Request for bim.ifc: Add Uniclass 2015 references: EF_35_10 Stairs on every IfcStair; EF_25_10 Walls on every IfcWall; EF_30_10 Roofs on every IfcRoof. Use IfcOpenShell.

First a look at what the model holds.

```python
import ifcopenshell

model = ifcopenshell.open("bim.ifc")
print(model.schema)
print("classifications:", [c.Name for c in model.by_type("IfcClassification")])
for ifc_class in ("IfcDoor", "IfcRoof", "IfcStair", "IfcWall", "IfcWindow"):
    print(ifc_class, len(model.by_type(ifc_class)))
```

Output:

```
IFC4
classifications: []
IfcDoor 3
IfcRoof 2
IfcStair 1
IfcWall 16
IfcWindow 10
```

```python
import ifcopenshell
import ifcopenshell.api.classification

model = ifcopenshell.open("bim.ifc")

system = ifcopenshell.api.classification.add_classification(model, classification="Uniclass 2015")

codes = {
    "IfcStair": ("EF_35_10", "Stairs"),
    "IfcWall": ("EF_25_10", "Walls"),
    "IfcRoof": ("EF_30_10", "Roofs"),
}
for ifc_class, (code, name) in codes.items():
    products = model.by_type(ifc_class)
    ifcopenshell.api.classification.add_reference(
        model, products=products, classification=system, identification=code, name=name
    )
    print(code, len(products))

model.write("bim-out.ifc")
```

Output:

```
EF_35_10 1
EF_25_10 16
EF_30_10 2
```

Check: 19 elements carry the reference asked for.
